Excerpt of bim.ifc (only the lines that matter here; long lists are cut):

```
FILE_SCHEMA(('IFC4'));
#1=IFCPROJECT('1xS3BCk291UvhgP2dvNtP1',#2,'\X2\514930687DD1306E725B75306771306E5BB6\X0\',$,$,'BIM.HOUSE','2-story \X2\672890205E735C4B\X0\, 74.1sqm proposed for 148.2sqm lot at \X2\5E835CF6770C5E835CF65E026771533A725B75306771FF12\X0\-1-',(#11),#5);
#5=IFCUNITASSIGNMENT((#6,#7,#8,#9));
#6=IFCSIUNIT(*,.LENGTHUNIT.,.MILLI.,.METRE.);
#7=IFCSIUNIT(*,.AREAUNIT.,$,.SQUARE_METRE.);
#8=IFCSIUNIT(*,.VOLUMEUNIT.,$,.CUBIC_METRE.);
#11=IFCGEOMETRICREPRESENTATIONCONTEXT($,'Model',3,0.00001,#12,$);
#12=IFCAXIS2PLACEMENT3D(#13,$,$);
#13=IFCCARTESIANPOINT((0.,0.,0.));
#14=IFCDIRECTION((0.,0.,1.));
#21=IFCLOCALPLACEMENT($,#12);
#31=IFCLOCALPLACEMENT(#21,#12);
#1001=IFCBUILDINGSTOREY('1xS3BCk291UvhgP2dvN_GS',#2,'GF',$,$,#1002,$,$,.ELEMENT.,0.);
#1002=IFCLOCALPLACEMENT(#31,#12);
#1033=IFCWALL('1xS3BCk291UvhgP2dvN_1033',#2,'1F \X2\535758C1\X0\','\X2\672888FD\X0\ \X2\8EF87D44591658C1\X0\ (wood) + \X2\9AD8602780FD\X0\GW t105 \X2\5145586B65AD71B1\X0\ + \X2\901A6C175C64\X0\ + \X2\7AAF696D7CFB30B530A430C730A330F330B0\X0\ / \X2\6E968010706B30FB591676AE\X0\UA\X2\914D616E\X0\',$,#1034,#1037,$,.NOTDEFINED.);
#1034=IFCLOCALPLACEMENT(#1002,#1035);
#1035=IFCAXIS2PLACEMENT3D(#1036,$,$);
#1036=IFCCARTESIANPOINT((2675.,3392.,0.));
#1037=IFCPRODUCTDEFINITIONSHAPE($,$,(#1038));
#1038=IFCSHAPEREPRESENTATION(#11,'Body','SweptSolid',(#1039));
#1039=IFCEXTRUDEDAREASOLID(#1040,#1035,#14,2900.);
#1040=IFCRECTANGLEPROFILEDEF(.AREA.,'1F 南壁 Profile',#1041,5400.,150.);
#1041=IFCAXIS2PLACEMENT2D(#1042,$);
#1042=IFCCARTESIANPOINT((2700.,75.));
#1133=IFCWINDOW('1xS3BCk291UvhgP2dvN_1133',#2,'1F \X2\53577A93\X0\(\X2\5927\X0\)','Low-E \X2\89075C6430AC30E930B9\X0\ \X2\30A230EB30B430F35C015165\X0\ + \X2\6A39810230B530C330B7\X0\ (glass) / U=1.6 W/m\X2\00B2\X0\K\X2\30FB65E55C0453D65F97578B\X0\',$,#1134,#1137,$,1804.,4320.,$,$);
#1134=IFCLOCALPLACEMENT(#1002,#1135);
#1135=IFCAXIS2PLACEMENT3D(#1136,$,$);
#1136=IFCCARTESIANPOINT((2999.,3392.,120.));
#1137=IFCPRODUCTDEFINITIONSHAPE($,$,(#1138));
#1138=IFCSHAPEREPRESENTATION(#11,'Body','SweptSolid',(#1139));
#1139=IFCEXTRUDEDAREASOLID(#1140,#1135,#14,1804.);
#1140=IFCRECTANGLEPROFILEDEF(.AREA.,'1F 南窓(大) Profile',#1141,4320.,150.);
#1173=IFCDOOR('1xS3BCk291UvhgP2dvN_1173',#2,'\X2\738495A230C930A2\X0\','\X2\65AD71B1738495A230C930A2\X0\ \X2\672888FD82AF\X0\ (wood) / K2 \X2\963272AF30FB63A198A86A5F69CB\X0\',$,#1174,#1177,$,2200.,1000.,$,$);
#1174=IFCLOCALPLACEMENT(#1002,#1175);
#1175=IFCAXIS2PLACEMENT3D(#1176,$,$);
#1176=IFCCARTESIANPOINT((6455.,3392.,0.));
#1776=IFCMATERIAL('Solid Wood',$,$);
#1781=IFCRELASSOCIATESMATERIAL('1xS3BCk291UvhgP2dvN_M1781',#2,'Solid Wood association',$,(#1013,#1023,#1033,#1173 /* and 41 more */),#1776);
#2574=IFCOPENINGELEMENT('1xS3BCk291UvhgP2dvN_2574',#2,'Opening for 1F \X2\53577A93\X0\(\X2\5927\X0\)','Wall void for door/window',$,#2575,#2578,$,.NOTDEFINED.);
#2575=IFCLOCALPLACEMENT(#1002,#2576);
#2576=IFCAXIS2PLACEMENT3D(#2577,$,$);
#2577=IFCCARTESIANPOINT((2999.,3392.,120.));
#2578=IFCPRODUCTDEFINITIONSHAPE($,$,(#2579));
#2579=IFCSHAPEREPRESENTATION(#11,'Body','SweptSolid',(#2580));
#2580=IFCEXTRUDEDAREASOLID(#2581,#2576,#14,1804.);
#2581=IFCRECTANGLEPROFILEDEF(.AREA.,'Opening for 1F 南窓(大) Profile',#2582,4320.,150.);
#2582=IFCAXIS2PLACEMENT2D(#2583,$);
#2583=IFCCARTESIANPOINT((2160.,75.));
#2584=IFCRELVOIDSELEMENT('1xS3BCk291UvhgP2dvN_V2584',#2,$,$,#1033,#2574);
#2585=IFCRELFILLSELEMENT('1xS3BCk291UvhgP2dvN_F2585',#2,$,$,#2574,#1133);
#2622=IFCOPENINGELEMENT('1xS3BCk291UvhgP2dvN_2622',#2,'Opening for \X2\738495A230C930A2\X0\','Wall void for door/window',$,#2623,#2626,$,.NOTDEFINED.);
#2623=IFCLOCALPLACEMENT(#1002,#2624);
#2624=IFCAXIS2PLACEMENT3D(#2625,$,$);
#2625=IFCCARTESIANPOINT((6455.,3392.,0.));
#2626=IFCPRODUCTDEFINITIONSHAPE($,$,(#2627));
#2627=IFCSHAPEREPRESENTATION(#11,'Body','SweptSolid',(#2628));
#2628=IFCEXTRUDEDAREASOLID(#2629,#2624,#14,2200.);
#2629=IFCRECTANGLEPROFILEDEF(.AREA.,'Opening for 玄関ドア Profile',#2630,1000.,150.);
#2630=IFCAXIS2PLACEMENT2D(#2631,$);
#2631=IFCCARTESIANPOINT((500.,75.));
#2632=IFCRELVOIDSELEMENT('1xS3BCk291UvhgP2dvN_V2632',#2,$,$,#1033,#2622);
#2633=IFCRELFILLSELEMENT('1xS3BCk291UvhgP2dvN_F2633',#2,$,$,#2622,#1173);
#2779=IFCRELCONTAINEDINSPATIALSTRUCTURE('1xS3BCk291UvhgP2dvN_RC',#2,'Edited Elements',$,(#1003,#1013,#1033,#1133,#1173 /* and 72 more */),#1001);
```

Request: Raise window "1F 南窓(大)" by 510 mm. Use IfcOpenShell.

```python
import numpy as np
import ifcopenshell
import ifcopenshell.api.geometry
import ifcopenshell.util.placement
import ifcopenshell.util.unit

model = ifcopenshell.open("bim.ifc")
unit_scale = ifcopenshell.util.unit.calculate_unit_scale(model)

window = model.by_guid("1xS3BCk291UvhgP2dvN_1133")
opening = window.FillsVoids[0].RelatingOpeningElement
dz = 0.51 / unit_scale

shift = np.array([0.0, 0.0, dz])
# The window is not placed relative to its opening, so move both.
for product in (opening, window):
    matrix = ifcopenshell.util.placement.get_local_placement(product.ObjectPlacement)
    matrix[:3, 3] += shift
    ifcopenshell.api.geometry.edit_object_placement(model, product=product, matrix=matrix, is_si=False)

print(f"moved by {dz * unit_scale:+.3f} m")

model.write("bim_updated.ifc")
```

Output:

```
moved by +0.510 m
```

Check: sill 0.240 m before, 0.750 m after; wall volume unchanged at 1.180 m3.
